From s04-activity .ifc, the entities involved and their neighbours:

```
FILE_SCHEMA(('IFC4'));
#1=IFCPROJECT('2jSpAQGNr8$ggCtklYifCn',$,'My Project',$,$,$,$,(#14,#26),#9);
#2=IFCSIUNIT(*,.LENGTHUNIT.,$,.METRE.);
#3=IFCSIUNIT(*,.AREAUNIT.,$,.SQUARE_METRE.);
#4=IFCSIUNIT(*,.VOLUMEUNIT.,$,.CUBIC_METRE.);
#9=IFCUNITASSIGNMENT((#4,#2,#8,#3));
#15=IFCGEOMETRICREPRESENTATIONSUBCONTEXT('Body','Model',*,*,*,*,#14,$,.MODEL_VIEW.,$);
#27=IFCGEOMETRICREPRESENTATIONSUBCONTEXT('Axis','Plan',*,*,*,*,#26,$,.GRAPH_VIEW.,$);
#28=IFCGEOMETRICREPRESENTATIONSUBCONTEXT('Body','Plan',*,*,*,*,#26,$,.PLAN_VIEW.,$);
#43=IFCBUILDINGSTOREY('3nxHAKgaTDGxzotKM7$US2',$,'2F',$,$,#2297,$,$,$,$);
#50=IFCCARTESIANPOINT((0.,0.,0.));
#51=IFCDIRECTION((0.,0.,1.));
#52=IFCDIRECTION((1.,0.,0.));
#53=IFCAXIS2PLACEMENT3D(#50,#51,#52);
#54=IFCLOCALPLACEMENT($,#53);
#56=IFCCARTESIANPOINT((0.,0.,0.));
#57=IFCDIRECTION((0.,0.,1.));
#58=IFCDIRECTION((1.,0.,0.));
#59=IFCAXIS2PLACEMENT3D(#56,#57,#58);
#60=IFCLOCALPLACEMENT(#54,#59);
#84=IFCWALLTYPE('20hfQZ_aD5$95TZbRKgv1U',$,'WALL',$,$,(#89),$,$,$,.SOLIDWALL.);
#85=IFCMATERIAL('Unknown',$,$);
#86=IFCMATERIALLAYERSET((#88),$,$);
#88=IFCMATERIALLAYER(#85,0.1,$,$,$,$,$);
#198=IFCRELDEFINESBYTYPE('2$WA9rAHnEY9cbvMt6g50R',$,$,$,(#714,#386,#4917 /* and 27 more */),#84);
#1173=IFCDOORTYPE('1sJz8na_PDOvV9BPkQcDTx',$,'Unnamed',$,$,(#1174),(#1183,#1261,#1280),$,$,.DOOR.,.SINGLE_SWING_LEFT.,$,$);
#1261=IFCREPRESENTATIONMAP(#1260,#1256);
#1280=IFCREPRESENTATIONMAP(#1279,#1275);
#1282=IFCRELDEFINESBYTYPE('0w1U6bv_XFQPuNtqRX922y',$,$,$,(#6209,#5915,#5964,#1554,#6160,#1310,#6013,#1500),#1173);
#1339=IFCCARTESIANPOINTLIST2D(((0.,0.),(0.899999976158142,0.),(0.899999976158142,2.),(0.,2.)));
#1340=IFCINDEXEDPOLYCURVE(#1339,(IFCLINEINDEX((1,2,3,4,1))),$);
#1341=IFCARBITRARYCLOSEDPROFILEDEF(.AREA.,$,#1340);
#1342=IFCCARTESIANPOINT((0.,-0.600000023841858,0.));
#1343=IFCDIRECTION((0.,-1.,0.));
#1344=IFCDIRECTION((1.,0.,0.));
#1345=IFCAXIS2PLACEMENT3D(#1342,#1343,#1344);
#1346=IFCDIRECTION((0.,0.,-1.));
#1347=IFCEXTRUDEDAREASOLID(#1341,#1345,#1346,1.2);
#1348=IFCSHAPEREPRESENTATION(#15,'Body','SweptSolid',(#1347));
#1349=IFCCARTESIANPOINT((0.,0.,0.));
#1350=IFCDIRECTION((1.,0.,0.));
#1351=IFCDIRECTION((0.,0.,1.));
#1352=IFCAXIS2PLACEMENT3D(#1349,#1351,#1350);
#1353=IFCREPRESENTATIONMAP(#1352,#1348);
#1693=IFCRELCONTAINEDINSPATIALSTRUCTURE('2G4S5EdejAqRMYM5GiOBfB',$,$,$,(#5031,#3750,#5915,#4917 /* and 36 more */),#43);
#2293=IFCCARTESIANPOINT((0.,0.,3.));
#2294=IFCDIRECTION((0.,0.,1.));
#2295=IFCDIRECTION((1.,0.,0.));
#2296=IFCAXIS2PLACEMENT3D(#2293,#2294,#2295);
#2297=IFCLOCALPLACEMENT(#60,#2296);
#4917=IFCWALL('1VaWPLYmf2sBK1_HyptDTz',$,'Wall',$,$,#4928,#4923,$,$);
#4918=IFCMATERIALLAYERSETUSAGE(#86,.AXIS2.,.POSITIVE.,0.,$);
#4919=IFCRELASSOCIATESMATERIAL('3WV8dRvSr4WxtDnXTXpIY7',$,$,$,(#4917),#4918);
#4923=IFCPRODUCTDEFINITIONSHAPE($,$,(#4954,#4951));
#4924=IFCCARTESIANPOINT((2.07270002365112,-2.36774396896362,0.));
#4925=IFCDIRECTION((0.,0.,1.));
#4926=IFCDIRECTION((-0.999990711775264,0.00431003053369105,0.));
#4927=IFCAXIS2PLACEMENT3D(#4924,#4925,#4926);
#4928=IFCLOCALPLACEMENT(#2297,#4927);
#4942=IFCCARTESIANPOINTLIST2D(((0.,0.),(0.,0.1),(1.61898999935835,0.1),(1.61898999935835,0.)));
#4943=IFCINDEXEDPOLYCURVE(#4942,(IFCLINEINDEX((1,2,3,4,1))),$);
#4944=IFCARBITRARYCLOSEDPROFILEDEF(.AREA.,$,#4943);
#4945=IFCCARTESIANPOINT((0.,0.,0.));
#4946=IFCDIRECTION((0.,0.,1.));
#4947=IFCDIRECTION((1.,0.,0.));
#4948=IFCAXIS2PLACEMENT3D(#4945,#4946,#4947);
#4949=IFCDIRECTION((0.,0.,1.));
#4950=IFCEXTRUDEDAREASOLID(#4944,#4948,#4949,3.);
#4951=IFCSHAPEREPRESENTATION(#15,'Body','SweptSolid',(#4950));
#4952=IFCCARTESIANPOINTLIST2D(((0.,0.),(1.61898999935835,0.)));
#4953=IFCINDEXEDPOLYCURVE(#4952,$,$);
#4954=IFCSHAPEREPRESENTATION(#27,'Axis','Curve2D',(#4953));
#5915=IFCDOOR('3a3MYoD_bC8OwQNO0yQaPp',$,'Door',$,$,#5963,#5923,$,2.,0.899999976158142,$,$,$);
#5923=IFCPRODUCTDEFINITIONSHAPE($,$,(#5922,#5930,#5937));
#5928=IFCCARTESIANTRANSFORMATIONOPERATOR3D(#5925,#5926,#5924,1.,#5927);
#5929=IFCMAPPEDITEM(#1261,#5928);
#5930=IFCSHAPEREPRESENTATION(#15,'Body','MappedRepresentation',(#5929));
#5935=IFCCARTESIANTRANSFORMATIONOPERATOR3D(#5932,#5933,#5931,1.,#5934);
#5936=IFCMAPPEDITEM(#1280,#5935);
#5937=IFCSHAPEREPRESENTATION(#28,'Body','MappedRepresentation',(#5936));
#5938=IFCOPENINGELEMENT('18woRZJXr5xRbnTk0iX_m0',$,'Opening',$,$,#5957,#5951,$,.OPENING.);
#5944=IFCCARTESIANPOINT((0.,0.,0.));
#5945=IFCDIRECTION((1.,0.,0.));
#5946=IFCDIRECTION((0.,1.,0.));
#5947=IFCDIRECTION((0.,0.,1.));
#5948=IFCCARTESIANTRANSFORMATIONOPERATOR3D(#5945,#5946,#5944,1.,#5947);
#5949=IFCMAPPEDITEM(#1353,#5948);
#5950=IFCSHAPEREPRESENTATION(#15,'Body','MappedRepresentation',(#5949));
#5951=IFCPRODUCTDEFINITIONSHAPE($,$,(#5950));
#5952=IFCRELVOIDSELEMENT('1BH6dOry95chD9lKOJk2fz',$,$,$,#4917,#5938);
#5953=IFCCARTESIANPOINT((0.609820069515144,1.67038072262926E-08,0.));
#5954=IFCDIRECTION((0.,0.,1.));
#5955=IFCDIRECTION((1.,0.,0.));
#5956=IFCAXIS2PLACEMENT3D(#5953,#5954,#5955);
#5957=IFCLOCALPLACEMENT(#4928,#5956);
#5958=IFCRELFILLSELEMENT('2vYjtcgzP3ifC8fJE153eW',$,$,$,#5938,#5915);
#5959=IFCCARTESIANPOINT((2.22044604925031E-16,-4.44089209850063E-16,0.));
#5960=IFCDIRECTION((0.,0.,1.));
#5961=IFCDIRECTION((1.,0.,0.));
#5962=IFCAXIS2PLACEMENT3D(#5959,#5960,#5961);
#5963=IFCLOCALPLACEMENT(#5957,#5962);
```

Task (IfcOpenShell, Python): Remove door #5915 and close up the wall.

```python
import ifcopenshell
import ifcopenshell.api.feature
import ifcopenshell.api.root
import ifcopenshell.geom
import ifcopenshell.util.shape

model = ifcopenshell.open("s04-activity .ifc")
settings = ifcopenshell.geom.settings()


def volume(element):
    """Net volume in cubic metres, openings subtracted."""
    shape = ifcopenshell.geom.create_shape(settings, element)
    return ifcopenshell.util.shape.get_volume(shape.geometry)


door = model.by_guid("3a3MYoD_bC8OwQNO0yQaPp")
opening = door.FillsVoids[0].RelatingOpeningElement
wall = opening.VoidsElements[0].RelatingBuildingElement
before = volume(wall)

ifcopenshell.api.root.remove_product(model, product=door)
ifcopenshell.api.feature.remove_feature(model, feature=opening)

after = volume(wall)

print(f"wall volume {before:.3f} -> {after:.3f} m3")

model.write("s04-activity _updated.ifc")
```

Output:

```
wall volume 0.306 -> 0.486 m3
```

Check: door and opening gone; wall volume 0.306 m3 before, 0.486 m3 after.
